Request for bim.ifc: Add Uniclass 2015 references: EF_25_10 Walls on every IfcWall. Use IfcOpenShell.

First a look at what the model holds.

```python
import ifcopenshell

model = ifcopenshell.open("bim.ifc")
print(model.schema)
print("classifications:", [c.Name for c in model.by_type("IfcClassification")])
for ifc_class in ("IfcDoor", "IfcRoof", "IfcStair", "IfcWall", "IfcWindow"):
    print(ifc_class, len(model.by_type(ifc_class)))
```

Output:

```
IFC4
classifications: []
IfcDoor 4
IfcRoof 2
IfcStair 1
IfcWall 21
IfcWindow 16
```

```python
import ifcopenshell
import ifcopenshell.api.classification

model = ifcopenshell.open("bim.ifc")

system = ifcopenshell.api.classification.add_classification(model, classification="Uniclass 2015")

codes = {
    "IfcWall": ("EF_25_10", "Walls"),
}
for ifc_class, (code, name) in codes.items():
    products = model.by_type(ifc_class)
    ifcopenshell.api.classification.add_reference(
        model, products=products, classification=system, identification=code, name=name
    )
    print(code, len(products))

model.write("bim-out.ifc")
```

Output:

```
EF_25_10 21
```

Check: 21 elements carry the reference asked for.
